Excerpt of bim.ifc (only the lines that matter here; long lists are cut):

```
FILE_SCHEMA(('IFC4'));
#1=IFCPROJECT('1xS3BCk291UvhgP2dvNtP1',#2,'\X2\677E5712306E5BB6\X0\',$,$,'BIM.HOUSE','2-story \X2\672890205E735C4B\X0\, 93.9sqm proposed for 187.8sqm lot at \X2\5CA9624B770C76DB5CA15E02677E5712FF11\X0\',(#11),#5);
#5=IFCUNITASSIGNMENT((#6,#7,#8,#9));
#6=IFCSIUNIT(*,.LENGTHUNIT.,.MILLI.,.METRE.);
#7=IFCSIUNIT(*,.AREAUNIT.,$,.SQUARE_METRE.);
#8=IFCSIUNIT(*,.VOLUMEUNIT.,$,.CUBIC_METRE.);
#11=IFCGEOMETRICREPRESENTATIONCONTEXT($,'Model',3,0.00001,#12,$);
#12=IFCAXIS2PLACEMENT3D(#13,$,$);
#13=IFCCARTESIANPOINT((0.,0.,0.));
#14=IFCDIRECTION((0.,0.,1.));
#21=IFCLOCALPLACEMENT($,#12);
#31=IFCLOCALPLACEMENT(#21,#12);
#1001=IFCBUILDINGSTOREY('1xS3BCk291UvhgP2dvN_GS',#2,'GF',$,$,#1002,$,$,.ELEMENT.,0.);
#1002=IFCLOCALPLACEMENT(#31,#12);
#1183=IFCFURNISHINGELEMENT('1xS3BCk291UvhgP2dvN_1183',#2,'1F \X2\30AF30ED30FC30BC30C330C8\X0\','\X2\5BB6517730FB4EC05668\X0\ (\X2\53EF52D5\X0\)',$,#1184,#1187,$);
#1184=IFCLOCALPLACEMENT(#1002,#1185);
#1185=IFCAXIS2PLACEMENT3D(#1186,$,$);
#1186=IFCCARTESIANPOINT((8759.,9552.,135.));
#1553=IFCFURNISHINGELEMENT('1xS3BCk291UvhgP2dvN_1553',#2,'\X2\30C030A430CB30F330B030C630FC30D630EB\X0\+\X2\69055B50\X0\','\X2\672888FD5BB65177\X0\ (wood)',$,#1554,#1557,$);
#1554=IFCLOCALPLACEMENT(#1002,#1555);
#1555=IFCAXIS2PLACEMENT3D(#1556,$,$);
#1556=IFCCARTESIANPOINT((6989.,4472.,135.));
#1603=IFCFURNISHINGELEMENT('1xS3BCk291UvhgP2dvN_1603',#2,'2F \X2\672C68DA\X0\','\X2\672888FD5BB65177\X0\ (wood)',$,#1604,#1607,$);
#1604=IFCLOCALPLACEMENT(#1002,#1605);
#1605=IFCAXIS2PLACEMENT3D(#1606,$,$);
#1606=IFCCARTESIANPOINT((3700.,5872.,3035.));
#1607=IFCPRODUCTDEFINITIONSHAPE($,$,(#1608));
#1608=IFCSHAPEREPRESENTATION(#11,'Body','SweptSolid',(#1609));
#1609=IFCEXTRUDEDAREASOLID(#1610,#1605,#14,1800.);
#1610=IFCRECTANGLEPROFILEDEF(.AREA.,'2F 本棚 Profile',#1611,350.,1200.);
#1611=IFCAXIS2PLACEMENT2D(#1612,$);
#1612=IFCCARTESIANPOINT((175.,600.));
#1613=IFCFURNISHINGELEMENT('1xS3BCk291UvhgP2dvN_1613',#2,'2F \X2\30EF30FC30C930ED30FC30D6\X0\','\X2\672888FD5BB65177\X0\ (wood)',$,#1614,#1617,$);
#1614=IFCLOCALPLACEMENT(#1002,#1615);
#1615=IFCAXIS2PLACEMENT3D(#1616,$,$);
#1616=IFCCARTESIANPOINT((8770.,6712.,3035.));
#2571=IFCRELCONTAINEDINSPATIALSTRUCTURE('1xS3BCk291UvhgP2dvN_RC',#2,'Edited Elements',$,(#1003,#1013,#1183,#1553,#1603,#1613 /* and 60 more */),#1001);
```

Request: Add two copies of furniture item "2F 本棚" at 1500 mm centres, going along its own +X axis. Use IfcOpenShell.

```python
import ifcopenshell
import ifcopenshell.api.geometry
import ifcopenshell.api.root
import ifcopenshell.util.element
import ifcopenshell.util.placement
import ifcopenshell.util.unit

model = ifcopenshell.open("bim.ifc")
unit_scale = ifcopenshell.util.unit.calculate_unit_scale(model)


def reuse_history(source, copy):
    """copy_class also copies each property set's owner history, people and application; keep the originals."""
    for rel in copy.IsDefinedBy:
        if rel.is_a("IfcRelDefinesByProperties") and (history := rel.RelatingPropertyDefinition.OwnerHistory):
            rel.RelatingPropertyDefinition.OwnerHistory = source.OwnerHistory
            ifcopenshell.util.element.remove_deep2(model, history)


source = model.by_guid("1xS3BCk291UvhgP2dvN_1603")
base = ifcopenshell.util.placement.get_local_placement(source.ObjectPlacement)
step = base[:3, 0] * 1.5 / unit_scale

for i in range(1, 3):
    copy = ifcopenshell.api.root.copy_class(model, product=source)
    copy.Representation = ifcopenshell.util.element.copy_deep(
        model, source.Representation, exclude=["IfcGeometricRepresentationContext", "IfcRepresentationMap"]
    )
    reuse_history(source, copy)
    matrix = base.copy()
    matrix[:3, 3] += i * step
    print("added at", matrix[:3, 3].round(3) + 0.0)
    ifcopenshell.api.geometry.edit_object_placement(model, product=copy, matrix=matrix, is_si=False)

model.write("bim_edited.ifc")
```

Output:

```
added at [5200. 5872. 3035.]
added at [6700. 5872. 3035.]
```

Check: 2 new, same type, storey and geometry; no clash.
